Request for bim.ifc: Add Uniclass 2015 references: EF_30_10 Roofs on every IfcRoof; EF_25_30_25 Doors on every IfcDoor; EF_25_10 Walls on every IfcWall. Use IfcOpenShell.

First a look at what the model holds.

```python
import ifcopenshell

model = ifcopenshell.open("bim.ifc")
print(model.schema)
print("classifications:", [c.Name for c in model.by_type("IfcClassification")])
for ifc_class in ("IfcDoor", "IfcRoof", "IfcStair", "IfcWall", "IfcWindow"):
    print(ifc_class, len(model.by_type(ifc_class)))
```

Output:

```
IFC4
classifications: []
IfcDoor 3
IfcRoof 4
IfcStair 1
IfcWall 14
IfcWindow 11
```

```python
import ifcopenshell
import ifcopenshell.api.classification

model = ifcopenshell.open("bim.ifc")

system = ifcopenshell.api.classification.add_classification(model, classification="Uniclass 2015")

codes = {
    "IfcRoof": ("EF_30_10", "Roofs"),
    "IfcDoor": ("EF_25_30_25", "Doors"),
    "IfcWall": ("EF_25_10", "Walls"),
}
for ifc_class, (code, name) in codes.items():
    products = model.by_type(ifc_class)
    ifcopenshell.api.classification.add_reference(
        model, products=products, classification=system, identification=code, name=name
    )
    print(code, len(products))

model.write("bim_rev.ifc")
```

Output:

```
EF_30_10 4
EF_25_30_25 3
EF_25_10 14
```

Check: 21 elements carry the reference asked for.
